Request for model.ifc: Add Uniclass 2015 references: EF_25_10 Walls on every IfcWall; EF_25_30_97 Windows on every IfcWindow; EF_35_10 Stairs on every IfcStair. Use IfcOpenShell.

First a look at what the model holds.

```python
import ifcopenshell

model = ifcopenshell.open("model.ifc")
print(model.schema)
print("classifications:", [c.Name for c in model.by_type("IfcClassification")])
for ifc_class in ("IfcDoor", "IfcRoof", "IfcStair", "IfcWall", "IfcWindow"):
    print(ifc_class, len(model.by_type(ifc_class)))
```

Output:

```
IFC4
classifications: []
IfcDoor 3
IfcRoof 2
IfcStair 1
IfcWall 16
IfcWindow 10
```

```python
import ifcopenshell
import ifcopenshell.api.classification

model = ifcopenshell.open("model.ifc")

system = ifcopenshell.api.classification.add_classification(model, classification="Uniclass 2015")

codes = {
    "IfcWall": ("EF_25_10", "Walls"),
    "IfcWindow": ("EF_25_30_97", "Windows"),
    "IfcStair": ("EF_35_10", "Stairs"),
}
for ifc_class, (code, name) in codes.items():
    products = model.by_type(ifc_class)
    ifcopenshell.api.classification.add_reference(
        model, products=products, classification=system, identification=code, name=name
    )
    print(code, len(products))

model.write("model_rev.ifc")
```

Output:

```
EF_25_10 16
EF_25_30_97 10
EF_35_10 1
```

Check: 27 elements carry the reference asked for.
